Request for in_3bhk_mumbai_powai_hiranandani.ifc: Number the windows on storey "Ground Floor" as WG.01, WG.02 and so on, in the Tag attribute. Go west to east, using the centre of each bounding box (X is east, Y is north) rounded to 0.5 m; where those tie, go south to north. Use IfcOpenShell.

First a look at what the model holds.

```python
import ifcopenshell
import ifcopenshell.util.element
import ifcopenshell.util.placement

model = ifcopenshell.open("in_3bhk_mumbai_powai_hiranandani.ifc")
print(model.schema)
storey = next(s for s in model.by_type("IfcBuildingStorey") if s.Name == "Ground Floor")
windows = [e for e in ifcopenshell.util.element.get_decomposition(storey) if e.is_a("IfcWindow")]
for e in sorted(windows, key=lambda e: e.id()):
    origin = ifcopenshell.util.placement.get_local_placement(e.ObjectPlacement)[:3, 3]
    print(e.id(), e.Tag, e.Name, origin.round(2) + 0.0, sep=" | ")
```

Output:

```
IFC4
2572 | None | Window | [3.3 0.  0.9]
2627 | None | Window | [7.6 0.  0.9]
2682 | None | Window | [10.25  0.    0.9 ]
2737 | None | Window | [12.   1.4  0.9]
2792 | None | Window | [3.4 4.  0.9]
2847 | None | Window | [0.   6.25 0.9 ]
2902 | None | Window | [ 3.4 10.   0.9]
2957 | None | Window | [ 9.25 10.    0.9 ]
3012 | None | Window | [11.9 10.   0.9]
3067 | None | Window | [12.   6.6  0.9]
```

```python
import ifcopenshell
import ifcopenshell.geom
import ifcopenshell.util.element
import ifcopenshell.util.shape

model = ifcopenshell.open("in_3bhk_mumbai_powai_hiranandani.ifc")
settings = ifcopenshell.geom.settings()
settings.set("use-world-coords", True)


def centre(element):
    shape = ifcopenshell.geom.create_shape(settings, element)
    return ifcopenshell.util.shape.get_bbox_centroid(shape.geometry)


storey = next(s for s in model.by_type("IfcBuildingStorey") if s.Name == "Ground Floor")
windows = [e for e in ifcopenshell.util.element.get_decomposition(storey) if e.is_a("IfcWindow")]

# Insertion points can sit at a corner or the storey origin, so sort by the geometry (in metres).
centres = {e: centre(e) for e in windows}
windows.sort(key=lambda e: (round(centres[e][0] / 0.5), centres[e][1]))

for i, e in enumerate(windows, start=1):
    number = f"WG.{i:02d}"
    e.Tag = number
    print(e.id(), number)

model.write("in_3bhk_mumbai_powai_hiranandani_v2.ifc")
```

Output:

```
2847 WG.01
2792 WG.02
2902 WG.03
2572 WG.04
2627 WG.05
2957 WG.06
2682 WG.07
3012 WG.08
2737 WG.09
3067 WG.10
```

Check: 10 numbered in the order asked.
